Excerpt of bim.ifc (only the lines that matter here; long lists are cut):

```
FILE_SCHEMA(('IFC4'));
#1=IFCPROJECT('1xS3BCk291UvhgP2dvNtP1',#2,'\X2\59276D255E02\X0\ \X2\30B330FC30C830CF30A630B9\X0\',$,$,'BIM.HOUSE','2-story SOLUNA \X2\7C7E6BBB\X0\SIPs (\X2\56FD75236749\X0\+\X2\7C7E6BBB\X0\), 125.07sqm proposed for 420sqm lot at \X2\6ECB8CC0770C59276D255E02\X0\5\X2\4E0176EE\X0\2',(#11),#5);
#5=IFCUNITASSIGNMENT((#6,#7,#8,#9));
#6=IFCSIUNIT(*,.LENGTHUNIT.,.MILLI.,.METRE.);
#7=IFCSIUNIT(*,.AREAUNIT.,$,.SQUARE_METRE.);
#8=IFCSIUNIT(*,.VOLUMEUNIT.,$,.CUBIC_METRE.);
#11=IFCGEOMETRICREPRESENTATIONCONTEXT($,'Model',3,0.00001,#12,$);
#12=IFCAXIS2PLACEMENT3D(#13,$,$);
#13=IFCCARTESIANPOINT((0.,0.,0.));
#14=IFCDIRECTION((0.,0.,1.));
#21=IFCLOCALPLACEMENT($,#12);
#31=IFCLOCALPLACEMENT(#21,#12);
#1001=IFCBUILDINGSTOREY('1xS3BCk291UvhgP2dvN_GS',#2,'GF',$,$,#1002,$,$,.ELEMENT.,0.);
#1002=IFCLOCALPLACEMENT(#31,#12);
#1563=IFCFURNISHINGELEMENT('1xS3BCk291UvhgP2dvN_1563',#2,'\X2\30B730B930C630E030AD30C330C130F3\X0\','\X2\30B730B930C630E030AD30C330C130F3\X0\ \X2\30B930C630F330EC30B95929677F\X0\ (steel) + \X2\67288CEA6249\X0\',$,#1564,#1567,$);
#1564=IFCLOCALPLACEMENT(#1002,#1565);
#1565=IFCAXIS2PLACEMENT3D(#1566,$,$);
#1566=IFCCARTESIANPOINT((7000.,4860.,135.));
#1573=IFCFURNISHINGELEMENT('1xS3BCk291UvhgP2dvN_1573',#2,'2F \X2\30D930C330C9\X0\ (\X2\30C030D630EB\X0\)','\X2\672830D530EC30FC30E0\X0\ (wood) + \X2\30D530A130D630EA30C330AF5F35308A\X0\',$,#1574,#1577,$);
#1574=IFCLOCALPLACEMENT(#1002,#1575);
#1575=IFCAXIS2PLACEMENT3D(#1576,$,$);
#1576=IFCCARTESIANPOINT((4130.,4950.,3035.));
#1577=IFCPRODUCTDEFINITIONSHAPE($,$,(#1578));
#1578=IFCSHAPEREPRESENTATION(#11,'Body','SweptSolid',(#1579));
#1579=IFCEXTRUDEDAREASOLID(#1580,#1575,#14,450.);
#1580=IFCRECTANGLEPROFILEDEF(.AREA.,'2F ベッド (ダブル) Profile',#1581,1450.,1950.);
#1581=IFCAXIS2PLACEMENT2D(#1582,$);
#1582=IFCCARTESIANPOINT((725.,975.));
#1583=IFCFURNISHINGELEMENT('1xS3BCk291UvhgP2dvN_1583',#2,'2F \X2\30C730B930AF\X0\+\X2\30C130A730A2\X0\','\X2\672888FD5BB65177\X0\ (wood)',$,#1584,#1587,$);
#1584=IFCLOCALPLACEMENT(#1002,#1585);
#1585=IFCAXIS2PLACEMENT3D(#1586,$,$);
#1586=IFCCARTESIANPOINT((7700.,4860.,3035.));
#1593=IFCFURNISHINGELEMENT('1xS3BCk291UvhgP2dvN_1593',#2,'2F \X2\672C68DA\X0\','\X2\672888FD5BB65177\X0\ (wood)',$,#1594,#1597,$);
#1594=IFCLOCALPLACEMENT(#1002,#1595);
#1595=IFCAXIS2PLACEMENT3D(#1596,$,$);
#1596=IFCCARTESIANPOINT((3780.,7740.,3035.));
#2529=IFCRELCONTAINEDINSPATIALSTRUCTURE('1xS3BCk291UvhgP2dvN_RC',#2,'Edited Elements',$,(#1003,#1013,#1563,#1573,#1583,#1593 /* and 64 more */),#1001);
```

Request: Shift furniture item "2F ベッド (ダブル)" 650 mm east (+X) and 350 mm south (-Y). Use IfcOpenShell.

```python
import ifcopenshell
import ifcopenshell.api.geometry
import ifcopenshell.util.placement
import ifcopenshell.util.unit

model = ifcopenshell.open("bim.ifc")
unit_scale = ifcopenshell.util.unit.calculate_unit_scale(model)

item = model.by_guid("1xS3BCk291UvhgP2dvN_1573")
matrix = ifcopenshell.util.placement.get_local_placement(item.ObjectPlacement)
matrix[0, 3] += 0.65 / unit_scale
matrix[1, 3] -= 0.35 / unit_scale
ifcopenshell.api.geometry.edit_object_placement(model, product=item, matrix=matrix, is_si=False)

print(ifcopenshell.util.placement.get_local_placement(item.ObjectPlacement).round(3) + 0.0)

model.write("bim_rev.ifc")
```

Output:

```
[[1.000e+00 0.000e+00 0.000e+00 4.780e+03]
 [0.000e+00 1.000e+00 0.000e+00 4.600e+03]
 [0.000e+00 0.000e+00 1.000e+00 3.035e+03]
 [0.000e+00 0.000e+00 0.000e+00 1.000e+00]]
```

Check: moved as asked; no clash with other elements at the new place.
